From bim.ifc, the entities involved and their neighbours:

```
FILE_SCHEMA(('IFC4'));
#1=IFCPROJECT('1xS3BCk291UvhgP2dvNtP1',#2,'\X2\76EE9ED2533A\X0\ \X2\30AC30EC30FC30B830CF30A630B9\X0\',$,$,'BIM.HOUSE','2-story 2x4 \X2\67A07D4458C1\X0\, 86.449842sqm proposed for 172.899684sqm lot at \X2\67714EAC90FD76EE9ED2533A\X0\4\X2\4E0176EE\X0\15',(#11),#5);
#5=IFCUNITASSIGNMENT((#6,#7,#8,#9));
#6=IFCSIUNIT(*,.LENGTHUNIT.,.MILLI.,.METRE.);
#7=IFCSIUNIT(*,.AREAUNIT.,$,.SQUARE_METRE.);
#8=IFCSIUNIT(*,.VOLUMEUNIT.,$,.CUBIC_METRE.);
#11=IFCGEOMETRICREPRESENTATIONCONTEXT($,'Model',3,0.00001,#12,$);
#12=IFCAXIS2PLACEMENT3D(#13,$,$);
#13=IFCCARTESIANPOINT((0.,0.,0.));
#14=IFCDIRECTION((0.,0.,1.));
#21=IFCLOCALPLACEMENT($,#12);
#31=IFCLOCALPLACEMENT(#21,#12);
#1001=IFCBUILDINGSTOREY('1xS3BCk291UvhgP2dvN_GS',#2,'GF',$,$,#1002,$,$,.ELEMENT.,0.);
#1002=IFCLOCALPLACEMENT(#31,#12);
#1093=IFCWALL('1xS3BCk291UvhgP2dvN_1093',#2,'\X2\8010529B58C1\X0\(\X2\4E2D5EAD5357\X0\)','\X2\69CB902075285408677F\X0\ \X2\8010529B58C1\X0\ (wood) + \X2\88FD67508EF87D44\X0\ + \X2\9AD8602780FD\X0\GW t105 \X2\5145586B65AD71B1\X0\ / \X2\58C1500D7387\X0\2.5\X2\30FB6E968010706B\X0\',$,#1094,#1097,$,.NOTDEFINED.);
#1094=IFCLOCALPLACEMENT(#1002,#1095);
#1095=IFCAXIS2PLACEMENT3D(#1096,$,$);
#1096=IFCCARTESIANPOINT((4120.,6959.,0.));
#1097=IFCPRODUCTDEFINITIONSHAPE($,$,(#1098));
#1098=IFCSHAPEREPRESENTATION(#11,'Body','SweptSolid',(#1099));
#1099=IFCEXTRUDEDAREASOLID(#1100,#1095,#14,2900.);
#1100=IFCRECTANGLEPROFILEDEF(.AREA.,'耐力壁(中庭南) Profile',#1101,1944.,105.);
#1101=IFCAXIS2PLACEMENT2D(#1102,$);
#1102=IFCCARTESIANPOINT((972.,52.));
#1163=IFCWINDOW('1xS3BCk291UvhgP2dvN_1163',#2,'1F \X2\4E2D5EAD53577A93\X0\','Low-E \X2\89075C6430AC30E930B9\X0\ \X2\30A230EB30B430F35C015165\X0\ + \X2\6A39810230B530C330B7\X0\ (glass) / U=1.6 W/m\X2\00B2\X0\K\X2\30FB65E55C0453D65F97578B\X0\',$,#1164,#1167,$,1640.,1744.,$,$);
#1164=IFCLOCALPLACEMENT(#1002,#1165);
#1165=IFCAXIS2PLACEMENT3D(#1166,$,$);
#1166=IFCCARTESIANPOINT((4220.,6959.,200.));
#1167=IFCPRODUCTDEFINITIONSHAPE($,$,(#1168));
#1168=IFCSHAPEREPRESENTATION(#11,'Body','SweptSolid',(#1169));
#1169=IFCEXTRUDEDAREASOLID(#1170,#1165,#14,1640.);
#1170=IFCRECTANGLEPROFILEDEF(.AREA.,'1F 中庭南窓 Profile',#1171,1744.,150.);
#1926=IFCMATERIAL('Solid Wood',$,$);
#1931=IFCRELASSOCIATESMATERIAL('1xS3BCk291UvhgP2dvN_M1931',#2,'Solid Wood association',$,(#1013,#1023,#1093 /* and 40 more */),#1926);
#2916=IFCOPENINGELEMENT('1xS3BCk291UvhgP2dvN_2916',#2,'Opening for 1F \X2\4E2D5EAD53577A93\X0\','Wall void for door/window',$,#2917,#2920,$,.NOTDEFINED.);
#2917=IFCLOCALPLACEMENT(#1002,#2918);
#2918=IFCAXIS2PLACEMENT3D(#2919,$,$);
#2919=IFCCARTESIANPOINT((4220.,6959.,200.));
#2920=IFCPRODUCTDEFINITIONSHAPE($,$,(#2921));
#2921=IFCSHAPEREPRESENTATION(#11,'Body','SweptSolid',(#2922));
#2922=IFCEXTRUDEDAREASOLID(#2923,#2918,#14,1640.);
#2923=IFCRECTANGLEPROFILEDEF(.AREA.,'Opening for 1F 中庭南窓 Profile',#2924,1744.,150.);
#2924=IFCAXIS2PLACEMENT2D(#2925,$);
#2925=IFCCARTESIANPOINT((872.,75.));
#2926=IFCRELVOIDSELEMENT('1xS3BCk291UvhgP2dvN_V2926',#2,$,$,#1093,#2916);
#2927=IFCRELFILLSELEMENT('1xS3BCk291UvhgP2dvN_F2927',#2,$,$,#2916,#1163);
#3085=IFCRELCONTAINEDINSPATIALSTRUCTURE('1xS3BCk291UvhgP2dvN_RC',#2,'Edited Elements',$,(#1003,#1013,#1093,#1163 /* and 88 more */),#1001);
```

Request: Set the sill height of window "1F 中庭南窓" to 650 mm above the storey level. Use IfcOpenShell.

```python
import numpy as np
import ifcopenshell
import ifcopenshell.api.geometry
import ifcopenshell.geom
import ifcopenshell.util.element
import ifcopenshell.util.placement
import ifcopenshell.util.shape
import ifcopenshell.util.unit

model = ifcopenshell.open("bim.ifc")
unit_scale = ifcopenshell.util.unit.calculate_unit_scale(model)

window = model.by_guid("1xS3BCk291UvhgP2dvN_1163")
opening = window.FillsVoids[0].RelatingOpeningElement
storey = ifcopenshell.util.element.get_container(window, ifc_class="IfcBuildingStorey")
level = ifcopenshell.util.placement.get_local_placement(storey.ObjectPlacement)[2, 3]

# The opening's origin need not be at the sill, so measure its lowest point.
shape = ifcopenshell.geom.create_shape(ifcopenshell.geom.settings(), opening)
bottom = ifcopenshell.util.shape.get_shape_bottom_elevation(shape, shape.geometry) / unit_scale
dz = level + 0.65 / unit_scale - bottom

shift = np.array([0.0, 0.0, dz])
# The window is not placed relative to its opening, so move both.
for product in (opening, window):
    matrix = ifcopenshell.util.placement.get_local_placement(product.ObjectPlacement)
    matrix[:3, 3] += shift
    ifcopenshell.api.geometry.edit_object_placement(model, product=product, matrix=matrix, is_si=False)

print(f"moved by {dz * unit_scale:+.3f} m")

model.write("bim_rev.ifc")
```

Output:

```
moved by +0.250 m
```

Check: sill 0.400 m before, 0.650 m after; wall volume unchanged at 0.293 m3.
